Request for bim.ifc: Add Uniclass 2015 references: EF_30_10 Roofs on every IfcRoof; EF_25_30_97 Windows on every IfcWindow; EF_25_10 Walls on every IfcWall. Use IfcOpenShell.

First a look at what the model holds.

```python
import ifcopenshell

model = ifcopenshell.open("bim.ifc")
print(model.schema)
print("classifications:", [c.Name for c in model.by_type("IfcClassification")])
for ifc_class in ("IfcDoor", "IfcRoof", "IfcStair", "IfcWall", "IfcWindow"):
    print(ifc_class, len(model.by_type(ifc_class)))
```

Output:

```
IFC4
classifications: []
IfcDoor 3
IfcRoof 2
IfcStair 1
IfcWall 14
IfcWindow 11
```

```python
import ifcopenshell
import ifcopenshell.api.classification

model = ifcopenshell.open("bim.ifc")

system = ifcopenshell.api.classification.add_classification(model, classification="Uniclass 2015")

codes = {
    "IfcRoof": ("EF_30_10", "Roofs"),
    "IfcWindow": ("EF_25_30_97", "Windows"),
    "IfcWall": ("EF_25_10", "Walls"),
}
for ifc_class, (code, name) in codes.items():
    products = model.by_type(ifc_class)
    ifcopenshell.api.classification.add_reference(
        model, products=products, classification=system, identification=code, name=name
    )
    print(code, len(products))

model.write("bim_v2.ifc")
```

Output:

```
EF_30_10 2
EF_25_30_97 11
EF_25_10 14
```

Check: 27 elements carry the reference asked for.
